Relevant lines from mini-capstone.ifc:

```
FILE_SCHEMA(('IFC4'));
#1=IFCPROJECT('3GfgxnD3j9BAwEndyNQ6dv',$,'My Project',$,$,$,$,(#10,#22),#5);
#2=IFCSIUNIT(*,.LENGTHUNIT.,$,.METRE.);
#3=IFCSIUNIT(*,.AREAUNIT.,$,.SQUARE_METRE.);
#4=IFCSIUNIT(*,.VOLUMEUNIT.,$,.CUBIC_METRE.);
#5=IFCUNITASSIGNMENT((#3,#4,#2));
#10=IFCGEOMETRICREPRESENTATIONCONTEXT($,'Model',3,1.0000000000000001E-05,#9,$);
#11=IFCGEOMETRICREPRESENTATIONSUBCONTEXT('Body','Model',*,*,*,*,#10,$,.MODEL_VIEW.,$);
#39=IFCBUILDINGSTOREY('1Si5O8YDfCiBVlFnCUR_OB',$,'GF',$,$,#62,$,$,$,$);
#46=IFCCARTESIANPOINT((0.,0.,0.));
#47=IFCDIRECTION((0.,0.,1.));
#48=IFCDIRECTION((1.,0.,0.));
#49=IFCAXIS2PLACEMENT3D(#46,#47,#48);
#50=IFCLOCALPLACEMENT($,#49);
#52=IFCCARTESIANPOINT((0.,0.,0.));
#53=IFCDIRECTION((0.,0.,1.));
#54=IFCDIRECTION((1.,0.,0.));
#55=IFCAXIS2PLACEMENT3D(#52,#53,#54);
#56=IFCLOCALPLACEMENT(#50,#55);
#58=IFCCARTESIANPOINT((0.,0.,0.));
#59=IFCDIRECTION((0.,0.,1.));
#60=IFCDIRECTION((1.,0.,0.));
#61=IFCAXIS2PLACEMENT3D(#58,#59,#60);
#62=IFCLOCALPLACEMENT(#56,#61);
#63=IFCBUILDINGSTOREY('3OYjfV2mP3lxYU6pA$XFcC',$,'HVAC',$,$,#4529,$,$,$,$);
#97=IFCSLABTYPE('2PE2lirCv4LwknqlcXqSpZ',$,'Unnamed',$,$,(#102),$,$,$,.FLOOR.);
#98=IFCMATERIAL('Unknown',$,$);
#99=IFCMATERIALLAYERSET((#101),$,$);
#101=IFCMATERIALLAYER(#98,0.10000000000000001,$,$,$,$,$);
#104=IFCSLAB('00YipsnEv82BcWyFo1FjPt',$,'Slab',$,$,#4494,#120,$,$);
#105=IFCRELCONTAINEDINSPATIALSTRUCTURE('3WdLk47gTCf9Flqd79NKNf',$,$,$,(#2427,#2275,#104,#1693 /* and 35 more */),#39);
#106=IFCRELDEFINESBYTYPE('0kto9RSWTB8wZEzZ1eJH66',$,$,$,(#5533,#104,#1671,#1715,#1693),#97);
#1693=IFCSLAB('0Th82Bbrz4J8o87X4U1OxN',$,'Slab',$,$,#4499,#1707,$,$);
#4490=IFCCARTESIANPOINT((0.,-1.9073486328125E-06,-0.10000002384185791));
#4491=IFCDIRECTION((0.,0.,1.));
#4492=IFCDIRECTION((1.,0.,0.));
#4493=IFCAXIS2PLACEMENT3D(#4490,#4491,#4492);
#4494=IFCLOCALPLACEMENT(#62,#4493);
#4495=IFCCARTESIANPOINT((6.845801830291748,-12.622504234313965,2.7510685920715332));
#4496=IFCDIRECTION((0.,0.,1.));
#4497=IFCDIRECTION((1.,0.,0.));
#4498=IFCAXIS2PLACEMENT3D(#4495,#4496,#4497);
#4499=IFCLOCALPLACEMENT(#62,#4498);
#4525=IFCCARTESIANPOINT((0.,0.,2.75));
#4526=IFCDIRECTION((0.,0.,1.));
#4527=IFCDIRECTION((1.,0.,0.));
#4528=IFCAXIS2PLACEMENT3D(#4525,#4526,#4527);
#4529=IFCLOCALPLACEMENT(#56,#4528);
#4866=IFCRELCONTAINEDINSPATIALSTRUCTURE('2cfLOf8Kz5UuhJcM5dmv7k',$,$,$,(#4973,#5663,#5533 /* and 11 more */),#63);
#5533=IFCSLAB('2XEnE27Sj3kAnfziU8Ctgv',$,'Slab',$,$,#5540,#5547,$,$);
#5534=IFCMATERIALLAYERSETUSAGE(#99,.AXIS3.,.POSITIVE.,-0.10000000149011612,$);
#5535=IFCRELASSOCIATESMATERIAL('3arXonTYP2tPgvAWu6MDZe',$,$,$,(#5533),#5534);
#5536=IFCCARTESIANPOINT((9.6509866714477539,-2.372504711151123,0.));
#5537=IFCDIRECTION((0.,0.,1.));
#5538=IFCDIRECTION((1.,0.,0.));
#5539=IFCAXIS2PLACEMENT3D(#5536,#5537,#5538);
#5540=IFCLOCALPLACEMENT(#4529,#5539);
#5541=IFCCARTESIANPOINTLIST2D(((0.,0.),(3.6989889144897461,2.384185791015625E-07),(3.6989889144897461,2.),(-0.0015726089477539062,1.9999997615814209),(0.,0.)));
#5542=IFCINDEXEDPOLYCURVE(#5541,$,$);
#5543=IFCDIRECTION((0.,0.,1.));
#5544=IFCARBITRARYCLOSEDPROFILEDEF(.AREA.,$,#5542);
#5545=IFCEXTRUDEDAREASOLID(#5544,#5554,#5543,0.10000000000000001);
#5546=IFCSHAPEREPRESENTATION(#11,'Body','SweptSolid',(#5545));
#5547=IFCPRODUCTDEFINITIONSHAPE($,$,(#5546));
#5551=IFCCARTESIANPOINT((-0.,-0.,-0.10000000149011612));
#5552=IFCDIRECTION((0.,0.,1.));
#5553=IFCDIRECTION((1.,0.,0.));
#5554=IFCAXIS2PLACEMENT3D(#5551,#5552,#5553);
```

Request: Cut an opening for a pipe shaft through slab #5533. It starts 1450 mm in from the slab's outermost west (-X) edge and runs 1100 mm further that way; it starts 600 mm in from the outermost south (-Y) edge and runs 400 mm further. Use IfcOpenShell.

```python
import numpy as np
import ifcopenshell
import ifcopenshell.api.feature
import ifcopenshell.api.geometry
import ifcopenshell.api.root
import ifcopenshell.geom
import ifcopenshell.util.placement
import ifcopenshell.util.representation
import ifcopenshell.util.shape
import ifcopenshell.util.unit

model = ifcopenshell.open("mini-capstone.ifc")
unit_scale = ifcopenshell.util.unit.calculate_unit_scale(model)
settings = ifcopenshell.geom.settings()


def volume(element):
    """Net volume in cubic metres, openings subtracted."""
    shape = ifcopenshell.geom.create_shape(settings, element)
    return ifcopenshell.util.shape.get_volume(shape.geometry)


slab = model.by_id(5533)
before = volume(slab)

# Extent in the slab's own axes, in metres. The edges named are its -X and -Y sides.
slab_shape = ifcopenshell.geom.create_shape(settings, slab)
vertices = ifcopenshell.util.shape.get_vertices(slab_shape.geometry)
x_min, y_min, bottom = vertices.min(axis=0)
top = vertices[:, 2].max()

opening = ifcopenshell.api.root.create_entity(model, ifc_class="IfcOpeningElement", name="Pipe shaft opening", predefined_type="OPENING")
context = ifcopenshell.util.representation.get_context(model, "Model", "Body", "MODEL_VIEW")
width, depth = 1.1, 0.4
outline = [(0.0, 0.0), (width, 0.0), (width, depth), (0.0, depth), (0.0, 0.0)]
# Overshoot both faces by 50 mm so the cut is clean.
shape = ifcopenshell.api.geometry.add_slab_representation(
    model, context=context, depth=top - bottom + 0.1, polyline=outline
)
ifcopenshell.api.geometry.assign_representation(model, product=opening, representation=shape)

matrix = ifcopenshell.util.placement.get_local_placement(slab.ObjectPlacement)
matrix[:, 3] = matrix @ np.append(np.array([x_min + 1.45, y_min + 0.6, bottom - 0.05]) / unit_scale, 1.0)
ifcopenshell.api.geometry.edit_object_placement(model, product=opening, matrix=matrix, is_si=False)
ifcopenshell.api.feature.add_feature(model, feature=opening, element=slab)

after = volume(slab)

print(f"slab volume {before:.3f} -> {after:.3f} m3")

model.write("mini-capstone_v2.ifc")
```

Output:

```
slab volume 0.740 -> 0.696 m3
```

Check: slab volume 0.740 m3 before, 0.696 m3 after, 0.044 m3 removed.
